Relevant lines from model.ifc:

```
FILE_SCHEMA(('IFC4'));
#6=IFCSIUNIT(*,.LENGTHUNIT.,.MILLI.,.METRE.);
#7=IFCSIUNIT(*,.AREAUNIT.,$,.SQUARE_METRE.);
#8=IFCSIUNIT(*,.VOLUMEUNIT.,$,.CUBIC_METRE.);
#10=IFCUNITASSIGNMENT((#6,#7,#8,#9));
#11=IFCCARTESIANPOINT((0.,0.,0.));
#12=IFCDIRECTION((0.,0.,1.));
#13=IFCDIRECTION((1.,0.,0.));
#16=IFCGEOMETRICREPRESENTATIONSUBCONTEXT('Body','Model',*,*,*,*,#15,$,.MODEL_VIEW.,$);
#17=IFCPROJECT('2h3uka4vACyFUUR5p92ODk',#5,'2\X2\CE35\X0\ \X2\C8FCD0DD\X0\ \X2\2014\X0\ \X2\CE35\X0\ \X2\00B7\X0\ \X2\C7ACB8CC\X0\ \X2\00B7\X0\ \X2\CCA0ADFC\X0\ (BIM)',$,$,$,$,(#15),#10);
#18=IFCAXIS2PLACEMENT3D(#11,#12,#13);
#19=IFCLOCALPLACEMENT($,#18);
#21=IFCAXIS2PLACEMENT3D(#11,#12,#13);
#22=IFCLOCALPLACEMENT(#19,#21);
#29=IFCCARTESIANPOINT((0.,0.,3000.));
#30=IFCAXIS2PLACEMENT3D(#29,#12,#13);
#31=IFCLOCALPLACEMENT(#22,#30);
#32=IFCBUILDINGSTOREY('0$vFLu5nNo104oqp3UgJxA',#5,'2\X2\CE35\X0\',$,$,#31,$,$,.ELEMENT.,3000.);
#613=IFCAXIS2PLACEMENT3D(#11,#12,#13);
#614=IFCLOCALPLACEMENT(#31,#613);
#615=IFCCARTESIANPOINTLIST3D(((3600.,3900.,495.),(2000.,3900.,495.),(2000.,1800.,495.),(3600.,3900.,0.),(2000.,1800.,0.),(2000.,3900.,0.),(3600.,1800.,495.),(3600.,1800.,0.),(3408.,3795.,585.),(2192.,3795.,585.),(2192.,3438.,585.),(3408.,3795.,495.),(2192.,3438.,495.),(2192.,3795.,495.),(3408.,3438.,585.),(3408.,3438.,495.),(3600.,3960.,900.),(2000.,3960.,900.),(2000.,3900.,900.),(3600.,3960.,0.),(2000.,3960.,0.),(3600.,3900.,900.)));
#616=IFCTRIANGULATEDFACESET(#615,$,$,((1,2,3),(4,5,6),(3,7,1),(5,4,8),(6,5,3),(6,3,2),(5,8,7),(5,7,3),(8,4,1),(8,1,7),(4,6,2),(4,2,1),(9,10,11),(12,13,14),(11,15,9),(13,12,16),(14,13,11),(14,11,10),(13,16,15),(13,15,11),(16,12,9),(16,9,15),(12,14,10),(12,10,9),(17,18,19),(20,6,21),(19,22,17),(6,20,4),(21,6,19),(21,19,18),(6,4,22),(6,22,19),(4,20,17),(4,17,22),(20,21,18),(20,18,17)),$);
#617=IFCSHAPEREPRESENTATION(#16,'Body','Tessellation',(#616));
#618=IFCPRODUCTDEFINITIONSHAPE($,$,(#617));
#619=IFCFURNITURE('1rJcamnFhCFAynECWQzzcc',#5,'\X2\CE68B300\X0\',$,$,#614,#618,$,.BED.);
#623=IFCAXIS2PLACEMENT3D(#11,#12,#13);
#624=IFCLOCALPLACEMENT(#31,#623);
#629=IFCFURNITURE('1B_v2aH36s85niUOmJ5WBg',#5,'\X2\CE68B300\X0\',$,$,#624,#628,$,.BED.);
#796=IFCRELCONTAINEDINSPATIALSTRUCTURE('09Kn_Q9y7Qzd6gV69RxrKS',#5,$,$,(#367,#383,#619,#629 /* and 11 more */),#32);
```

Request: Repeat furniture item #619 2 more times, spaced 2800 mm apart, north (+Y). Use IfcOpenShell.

```python
import numpy as np
import ifcopenshell
import ifcopenshell.api.geometry
import ifcopenshell.api.root
import ifcopenshell.util.element
import ifcopenshell.util.placement

model = ifcopenshell.open("model.ifc")


def reuse_history(source, copy):
    """copy_class also copies each property set's owner history, people and application; keep the originals."""
    for rel in copy.IsDefinedBy:
        if rel.is_a("IfcRelDefinesByProperties") and (history := rel.RelatingPropertyDefinition.OwnerHistory):
            rel.RelatingPropertyDefinition.OwnerHistory = source.OwnerHistory
            ifcopenshell.util.element.remove_deep2(model, history)


source = model.by_id(619)
base = ifcopenshell.util.placement.get_local_placement(source.ObjectPlacement)
step = np.array([0.0, 1.0, 0.0]) * 2800.0

for i in range(1, 3):
    copy = ifcopenshell.api.root.copy_class(model, product=source)
    copy.Representation = ifcopenshell.util.element.copy_deep(
        model, source.Representation, exclude=["IfcGeometricRepresentationContext", "IfcRepresentationMap"]
    )
    reuse_history(source, copy)
    matrix = base.copy()
    matrix[:3, 3] += i * step
    print("added at", matrix[:3, 3].round(3) + 0.0)
    ifcopenshell.api.geometry.edit_object_placement(model, product=copy, matrix=matrix, is_si=False)

model.write("model_updated.ifc")
```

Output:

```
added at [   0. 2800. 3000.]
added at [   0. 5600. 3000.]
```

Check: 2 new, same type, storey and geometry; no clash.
